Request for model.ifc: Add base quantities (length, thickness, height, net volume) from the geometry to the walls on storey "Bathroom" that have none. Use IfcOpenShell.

First a look at what the model holds.

```python
import ifcopenshell
import ifcopenshell.util.element
import ifcopenshell.util.unit

model = ifcopenshell.open("model.ifc")
print(model.schema)
for unit_type in ("LENGTHUNIT", "AREAUNIT", "VOLUMEUNIT"):
    print(unit_type, ifcopenshell.util.unit.calculate_unit_scale(model, unit_type))
storey = next(s for s in model.by_type("IfcBuildingStorey") if s.Name == "Bathroom")
walls = [e for e in ifcopenshell.util.element.get_decomposition(storey) if e.is_a("IfcWall")]
for e in sorted(walls, key=lambda e: e.id()):
    print(e.id(), e.is_a(), e.Name, list(ifcopenshell.util.element.get_psets(e, qtos_only=True)), sep=" | ")
```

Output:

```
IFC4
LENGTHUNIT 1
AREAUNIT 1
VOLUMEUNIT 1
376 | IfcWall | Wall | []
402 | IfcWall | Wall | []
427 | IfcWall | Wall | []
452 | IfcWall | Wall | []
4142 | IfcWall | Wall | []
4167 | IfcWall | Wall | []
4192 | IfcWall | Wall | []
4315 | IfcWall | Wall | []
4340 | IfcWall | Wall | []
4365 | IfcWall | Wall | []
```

```python
import ifcopenshell
import ifcopenshell.api.pset
import ifcopenshell.geom
import ifcopenshell.util.element
import ifcopenshell.util.shape
import ifcopenshell.util.unit

model = ifcopenshell.open("model.ifc")
unit_scale = ifcopenshell.util.unit.calculate_unit_scale(model)
volume_scale = ifcopenshell.util.unit.calculate_unit_scale(model, "VOLUMEUNIT")
settings = ifcopenshell.geom.settings()

storey = next(s for s in model.by_type("IfcBuildingStorey") if s.Name == "Bathroom")
walls = [e for e in ifcopenshell.util.element.get_decomposition(storey) if e.is_a("IfcWall")]

for e in sorted(walls, key=lambda e: e.id()):
    if ifcopenshell.util.element.get_psets(e, qtos_only=True, should_inherit=False):
        continue
    # Geometry comes back in metres, in the element's own axes.
    shape = ifcopenshell.geom.create_shape(settings, e)
    values = {
        "Length": ifcopenshell.util.shape.get_x(shape.geometry) / unit_scale,
        "Width": ifcopenshell.util.shape.get_y(shape.geometry) / unit_scale,
        "Height": ifcopenshell.util.shape.get_z(shape.geometry) / unit_scale,
        "NetVolume": ifcopenshell.util.shape.get_volume(shape.geometry) / volume_scale,
    }
    qto = ifcopenshell.api.pset.add_qto(model, product=e, name="Qto_WallBaseQuantities")
    ifcopenshell.api.pset.edit_qto(model, qto=qto, properties=values)
    print(e.id(), {k: round(v, 3) for k, v in values.items()})

model.write("model_updated.ifc")
```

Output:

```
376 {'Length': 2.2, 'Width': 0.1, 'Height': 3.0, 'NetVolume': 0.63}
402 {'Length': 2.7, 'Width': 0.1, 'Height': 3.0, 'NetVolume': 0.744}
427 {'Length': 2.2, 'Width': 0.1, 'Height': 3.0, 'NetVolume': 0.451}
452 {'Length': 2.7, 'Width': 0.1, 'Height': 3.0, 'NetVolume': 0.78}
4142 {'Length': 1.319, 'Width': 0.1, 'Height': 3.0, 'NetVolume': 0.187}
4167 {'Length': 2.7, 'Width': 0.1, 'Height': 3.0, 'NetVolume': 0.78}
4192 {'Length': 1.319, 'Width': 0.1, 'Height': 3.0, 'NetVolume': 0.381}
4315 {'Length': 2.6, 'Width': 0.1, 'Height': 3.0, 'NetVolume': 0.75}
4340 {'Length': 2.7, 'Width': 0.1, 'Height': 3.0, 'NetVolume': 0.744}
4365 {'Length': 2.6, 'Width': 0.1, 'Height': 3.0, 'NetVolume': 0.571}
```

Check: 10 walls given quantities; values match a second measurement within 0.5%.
